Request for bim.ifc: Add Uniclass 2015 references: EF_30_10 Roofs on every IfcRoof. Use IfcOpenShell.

First a look at what the model holds.

```python
import ifcopenshell

model = ifcopenshell.open("bim.ifc")
print(model.schema)
print("classifications:", [c.Name for c in model.by_type("IfcClassification")])
for ifc_class in ("IfcDoor", "IfcRoof", "IfcStair", "IfcWall", "IfcWindow"):
    print(ifc_class, len(model.by_type(ifc_class)))
```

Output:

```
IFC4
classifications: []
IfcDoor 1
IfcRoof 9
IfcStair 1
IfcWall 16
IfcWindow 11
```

```python
import ifcopenshell
import ifcopenshell.api.classification

model = ifcopenshell.open("bim.ifc")

system = ifcopenshell.api.classification.add_classification(model, classification="Uniclass 2015")

codes = {
    "IfcRoof": ("EF_30_10", "Roofs"),
}
for ifc_class, (code, name) in codes.items():
    products = model.by_type(ifc_class)
    ifcopenshell.api.classification.add_reference(
        model, products=products, classification=system, identification=code, name=name
    )
    print(code, len(products))

model.write("bim_edited.ifc")
```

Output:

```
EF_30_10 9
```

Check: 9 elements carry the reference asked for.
